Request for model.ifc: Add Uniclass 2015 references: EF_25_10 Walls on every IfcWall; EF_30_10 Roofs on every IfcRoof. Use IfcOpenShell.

First a look at what the model holds.

```python
import ifcopenshell

model = ifcopenshell.open("model.ifc")
print(model.schema)
print("classifications:", [c.Name for c in model.by_type("IfcClassification")])
for ifc_class in ("IfcDoor", "IfcRoof", "IfcStair", "IfcWall", "IfcWindow"):
    print(ifc_class, len(model.by_type(ifc_class)))
```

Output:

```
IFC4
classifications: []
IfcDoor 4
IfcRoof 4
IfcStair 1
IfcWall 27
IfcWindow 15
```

```python
import ifcopenshell
import ifcopenshell.api.classification

model = ifcopenshell.open("model.ifc")

system = ifcopenshell.api.classification.add_classification(model, classification="Uniclass 2015")

codes = {
    "IfcWall": ("EF_25_10", "Walls"),
    "IfcRoof": ("EF_30_10", "Roofs"),
}
for ifc_class, (code, name) in codes.items():
    products = model.by_type(ifc_class)
    ifcopenshell.api.classification.add_reference(
        model, products=products, classification=system, identification=code, name=name
    )
    print(code, len(products))

model.write("model_rev.ifc")
```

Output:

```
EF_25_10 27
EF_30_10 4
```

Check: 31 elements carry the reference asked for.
